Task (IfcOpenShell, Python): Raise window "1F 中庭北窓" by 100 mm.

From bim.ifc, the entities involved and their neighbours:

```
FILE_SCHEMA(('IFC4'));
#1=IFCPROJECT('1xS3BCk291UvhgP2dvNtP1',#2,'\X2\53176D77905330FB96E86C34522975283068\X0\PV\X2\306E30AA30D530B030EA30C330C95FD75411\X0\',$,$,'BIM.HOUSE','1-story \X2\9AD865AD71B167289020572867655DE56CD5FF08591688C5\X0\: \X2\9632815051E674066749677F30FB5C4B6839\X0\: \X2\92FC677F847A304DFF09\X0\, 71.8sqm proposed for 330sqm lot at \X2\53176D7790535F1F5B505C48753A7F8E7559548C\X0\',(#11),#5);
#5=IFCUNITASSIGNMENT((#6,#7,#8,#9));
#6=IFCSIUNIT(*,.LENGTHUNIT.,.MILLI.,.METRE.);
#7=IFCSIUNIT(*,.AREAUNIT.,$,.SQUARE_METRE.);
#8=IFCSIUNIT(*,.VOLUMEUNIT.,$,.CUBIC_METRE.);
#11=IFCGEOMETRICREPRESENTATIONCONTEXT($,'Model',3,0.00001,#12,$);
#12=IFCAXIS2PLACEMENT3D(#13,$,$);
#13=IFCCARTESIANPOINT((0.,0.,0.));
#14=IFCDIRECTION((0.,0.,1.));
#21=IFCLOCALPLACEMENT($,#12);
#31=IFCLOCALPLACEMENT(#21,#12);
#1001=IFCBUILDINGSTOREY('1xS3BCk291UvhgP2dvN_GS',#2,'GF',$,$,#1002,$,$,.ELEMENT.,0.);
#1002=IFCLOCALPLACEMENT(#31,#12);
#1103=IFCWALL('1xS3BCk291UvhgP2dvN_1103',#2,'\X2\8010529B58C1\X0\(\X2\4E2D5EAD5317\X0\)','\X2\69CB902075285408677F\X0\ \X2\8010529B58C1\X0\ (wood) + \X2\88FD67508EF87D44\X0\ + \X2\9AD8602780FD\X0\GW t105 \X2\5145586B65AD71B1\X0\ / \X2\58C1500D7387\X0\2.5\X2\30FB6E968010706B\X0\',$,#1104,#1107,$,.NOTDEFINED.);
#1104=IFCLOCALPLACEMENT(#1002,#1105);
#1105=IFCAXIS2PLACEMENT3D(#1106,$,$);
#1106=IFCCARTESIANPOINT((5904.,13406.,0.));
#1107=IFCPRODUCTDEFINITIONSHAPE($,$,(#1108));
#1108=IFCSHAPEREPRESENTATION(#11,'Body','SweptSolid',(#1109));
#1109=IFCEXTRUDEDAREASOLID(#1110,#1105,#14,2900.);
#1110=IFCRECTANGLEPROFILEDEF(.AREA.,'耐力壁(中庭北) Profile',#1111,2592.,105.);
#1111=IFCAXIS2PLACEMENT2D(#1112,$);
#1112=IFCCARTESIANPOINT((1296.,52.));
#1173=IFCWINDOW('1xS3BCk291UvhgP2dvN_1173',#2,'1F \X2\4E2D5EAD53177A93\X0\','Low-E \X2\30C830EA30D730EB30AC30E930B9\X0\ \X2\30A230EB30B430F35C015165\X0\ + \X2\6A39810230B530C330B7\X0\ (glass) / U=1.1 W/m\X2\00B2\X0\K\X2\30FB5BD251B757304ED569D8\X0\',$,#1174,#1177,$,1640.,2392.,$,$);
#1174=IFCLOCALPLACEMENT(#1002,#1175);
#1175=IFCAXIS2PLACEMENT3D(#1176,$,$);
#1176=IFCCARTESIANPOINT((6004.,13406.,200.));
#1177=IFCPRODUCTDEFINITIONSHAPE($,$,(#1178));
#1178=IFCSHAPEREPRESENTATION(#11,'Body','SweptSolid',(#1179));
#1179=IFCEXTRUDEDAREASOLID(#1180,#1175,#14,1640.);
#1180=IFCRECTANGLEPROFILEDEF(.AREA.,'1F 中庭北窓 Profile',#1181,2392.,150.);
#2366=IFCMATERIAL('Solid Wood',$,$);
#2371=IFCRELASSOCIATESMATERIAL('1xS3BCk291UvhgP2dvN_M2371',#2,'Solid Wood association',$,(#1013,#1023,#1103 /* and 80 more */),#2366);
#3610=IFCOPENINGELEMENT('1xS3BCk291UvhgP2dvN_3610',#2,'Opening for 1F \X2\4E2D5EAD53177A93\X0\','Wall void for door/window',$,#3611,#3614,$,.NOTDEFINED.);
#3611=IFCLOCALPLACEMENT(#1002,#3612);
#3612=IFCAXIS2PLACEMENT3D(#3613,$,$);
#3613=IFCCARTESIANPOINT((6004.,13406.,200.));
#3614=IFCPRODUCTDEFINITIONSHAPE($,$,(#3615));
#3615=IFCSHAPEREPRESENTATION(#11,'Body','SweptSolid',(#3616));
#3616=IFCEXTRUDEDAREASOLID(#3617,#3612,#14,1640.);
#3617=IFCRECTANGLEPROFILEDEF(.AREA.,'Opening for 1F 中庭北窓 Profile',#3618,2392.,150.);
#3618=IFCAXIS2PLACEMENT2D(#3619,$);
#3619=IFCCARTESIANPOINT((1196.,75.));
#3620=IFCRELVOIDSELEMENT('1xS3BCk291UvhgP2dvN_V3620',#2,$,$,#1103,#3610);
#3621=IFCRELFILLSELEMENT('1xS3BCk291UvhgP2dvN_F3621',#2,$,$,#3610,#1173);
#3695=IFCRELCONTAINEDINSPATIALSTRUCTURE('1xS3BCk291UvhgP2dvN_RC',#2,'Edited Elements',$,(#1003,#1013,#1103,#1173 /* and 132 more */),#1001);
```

```python
import numpy as np
import ifcopenshell
import ifcopenshell.api.geometry
import ifcopenshell.util.placement
import ifcopenshell.util.unit

model = ifcopenshell.open("bim.ifc")
unit_scale = ifcopenshell.util.unit.calculate_unit_scale(model)

window = model.by_guid("1xS3BCk291UvhgP2dvN_1173")
opening = window.FillsVoids[0].RelatingOpeningElement
dz = 0.1 / unit_scale

shift = np.array([0.0, 0.0, dz])
# The window is not placed relative to its opening, so move both.
for product in (opening, window):
    matrix = ifcopenshell.util.placement.get_local_placement(product.ObjectPlacement)
    matrix[:3, 3] += shift
    ifcopenshell.api.geometry.edit_object_placement(model, product=product, matrix=matrix, is_si=False)

print(f"moved by {dz * unit_scale:+.3f} m")

model.write("bim_updated.ifc")
```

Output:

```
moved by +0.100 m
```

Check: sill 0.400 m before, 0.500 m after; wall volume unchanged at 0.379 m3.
